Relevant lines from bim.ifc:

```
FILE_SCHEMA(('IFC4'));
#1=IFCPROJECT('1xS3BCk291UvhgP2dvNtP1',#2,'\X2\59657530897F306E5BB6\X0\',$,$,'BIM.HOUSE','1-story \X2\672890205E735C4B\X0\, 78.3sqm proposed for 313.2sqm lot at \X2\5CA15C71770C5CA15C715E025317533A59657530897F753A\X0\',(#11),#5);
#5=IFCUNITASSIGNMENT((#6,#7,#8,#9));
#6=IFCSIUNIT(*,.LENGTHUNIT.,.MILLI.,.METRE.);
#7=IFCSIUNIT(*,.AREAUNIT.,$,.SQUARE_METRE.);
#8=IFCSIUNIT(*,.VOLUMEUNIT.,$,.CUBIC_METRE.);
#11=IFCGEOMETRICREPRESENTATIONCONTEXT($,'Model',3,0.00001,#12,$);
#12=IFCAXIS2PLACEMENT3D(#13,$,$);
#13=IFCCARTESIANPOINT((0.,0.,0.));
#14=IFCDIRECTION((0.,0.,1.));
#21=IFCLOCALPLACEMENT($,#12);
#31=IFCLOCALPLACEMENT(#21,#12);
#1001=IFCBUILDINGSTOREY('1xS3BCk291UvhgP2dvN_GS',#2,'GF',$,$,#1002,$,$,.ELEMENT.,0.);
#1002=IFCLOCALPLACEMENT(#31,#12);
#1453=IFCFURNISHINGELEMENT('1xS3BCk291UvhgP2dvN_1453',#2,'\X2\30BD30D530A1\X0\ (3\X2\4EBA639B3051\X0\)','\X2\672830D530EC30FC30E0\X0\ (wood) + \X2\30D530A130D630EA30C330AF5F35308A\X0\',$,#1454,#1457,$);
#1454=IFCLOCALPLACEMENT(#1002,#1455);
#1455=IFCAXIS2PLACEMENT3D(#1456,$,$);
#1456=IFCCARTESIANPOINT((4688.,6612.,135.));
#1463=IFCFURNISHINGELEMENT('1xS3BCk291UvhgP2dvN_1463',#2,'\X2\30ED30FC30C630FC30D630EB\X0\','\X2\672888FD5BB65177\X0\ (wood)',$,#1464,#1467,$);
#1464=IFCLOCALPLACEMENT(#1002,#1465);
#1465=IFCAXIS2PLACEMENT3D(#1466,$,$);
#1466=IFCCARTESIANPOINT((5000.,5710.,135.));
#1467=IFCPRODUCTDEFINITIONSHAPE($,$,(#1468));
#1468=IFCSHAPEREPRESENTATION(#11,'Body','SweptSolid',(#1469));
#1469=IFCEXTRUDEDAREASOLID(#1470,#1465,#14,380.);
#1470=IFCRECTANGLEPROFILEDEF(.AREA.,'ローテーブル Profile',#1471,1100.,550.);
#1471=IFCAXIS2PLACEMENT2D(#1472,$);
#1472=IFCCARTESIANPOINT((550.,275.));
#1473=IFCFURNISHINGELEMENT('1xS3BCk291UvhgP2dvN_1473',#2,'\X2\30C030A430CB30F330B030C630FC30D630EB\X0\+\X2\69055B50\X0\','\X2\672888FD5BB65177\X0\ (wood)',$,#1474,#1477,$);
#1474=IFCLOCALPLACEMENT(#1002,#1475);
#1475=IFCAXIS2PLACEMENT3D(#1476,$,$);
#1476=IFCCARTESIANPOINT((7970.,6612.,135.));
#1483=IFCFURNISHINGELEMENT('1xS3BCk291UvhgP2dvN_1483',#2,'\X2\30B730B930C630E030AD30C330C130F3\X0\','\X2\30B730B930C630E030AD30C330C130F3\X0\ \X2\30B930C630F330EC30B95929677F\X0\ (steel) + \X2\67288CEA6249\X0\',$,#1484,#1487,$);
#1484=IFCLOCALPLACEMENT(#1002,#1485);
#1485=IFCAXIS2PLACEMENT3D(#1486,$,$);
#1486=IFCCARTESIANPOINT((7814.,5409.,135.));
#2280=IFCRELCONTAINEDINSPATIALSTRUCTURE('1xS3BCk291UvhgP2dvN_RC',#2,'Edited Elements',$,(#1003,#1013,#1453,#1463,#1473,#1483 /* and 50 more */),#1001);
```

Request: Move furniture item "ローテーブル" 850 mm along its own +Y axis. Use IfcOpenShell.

```python
import ifcopenshell
import ifcopenshell.api.geometry
import ifcopenshell.util.placement
import ifcopenshell.util.unit

model = ifcopenshell.open("bim.ifc")
unit_scale = ifcopenshell.util.unit.calculate_unit_scale(model)

item = model.by_guid("1xS3BCk291UvhgP2dvN_1463")
matrix = ifcopenshell.util.placement.get_local_placement(item.ObjectPlacement)
matrix[:3, 3] += matrix[:3, 1] * 0.85 / unit_scale
ifcopenshell.api.geometry.edit_object_placement(model, product=item, matrix=matrix, is_si=False)

print(ifcopenshell.util.placement.get_local_placement(item.ObjectPlacement).round(3) + 0.0)

model.write("bim_updated.ifc")
```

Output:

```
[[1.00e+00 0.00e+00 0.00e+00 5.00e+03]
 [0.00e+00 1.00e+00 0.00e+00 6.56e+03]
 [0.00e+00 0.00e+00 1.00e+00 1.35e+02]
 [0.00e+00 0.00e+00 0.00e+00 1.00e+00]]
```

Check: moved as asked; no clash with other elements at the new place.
